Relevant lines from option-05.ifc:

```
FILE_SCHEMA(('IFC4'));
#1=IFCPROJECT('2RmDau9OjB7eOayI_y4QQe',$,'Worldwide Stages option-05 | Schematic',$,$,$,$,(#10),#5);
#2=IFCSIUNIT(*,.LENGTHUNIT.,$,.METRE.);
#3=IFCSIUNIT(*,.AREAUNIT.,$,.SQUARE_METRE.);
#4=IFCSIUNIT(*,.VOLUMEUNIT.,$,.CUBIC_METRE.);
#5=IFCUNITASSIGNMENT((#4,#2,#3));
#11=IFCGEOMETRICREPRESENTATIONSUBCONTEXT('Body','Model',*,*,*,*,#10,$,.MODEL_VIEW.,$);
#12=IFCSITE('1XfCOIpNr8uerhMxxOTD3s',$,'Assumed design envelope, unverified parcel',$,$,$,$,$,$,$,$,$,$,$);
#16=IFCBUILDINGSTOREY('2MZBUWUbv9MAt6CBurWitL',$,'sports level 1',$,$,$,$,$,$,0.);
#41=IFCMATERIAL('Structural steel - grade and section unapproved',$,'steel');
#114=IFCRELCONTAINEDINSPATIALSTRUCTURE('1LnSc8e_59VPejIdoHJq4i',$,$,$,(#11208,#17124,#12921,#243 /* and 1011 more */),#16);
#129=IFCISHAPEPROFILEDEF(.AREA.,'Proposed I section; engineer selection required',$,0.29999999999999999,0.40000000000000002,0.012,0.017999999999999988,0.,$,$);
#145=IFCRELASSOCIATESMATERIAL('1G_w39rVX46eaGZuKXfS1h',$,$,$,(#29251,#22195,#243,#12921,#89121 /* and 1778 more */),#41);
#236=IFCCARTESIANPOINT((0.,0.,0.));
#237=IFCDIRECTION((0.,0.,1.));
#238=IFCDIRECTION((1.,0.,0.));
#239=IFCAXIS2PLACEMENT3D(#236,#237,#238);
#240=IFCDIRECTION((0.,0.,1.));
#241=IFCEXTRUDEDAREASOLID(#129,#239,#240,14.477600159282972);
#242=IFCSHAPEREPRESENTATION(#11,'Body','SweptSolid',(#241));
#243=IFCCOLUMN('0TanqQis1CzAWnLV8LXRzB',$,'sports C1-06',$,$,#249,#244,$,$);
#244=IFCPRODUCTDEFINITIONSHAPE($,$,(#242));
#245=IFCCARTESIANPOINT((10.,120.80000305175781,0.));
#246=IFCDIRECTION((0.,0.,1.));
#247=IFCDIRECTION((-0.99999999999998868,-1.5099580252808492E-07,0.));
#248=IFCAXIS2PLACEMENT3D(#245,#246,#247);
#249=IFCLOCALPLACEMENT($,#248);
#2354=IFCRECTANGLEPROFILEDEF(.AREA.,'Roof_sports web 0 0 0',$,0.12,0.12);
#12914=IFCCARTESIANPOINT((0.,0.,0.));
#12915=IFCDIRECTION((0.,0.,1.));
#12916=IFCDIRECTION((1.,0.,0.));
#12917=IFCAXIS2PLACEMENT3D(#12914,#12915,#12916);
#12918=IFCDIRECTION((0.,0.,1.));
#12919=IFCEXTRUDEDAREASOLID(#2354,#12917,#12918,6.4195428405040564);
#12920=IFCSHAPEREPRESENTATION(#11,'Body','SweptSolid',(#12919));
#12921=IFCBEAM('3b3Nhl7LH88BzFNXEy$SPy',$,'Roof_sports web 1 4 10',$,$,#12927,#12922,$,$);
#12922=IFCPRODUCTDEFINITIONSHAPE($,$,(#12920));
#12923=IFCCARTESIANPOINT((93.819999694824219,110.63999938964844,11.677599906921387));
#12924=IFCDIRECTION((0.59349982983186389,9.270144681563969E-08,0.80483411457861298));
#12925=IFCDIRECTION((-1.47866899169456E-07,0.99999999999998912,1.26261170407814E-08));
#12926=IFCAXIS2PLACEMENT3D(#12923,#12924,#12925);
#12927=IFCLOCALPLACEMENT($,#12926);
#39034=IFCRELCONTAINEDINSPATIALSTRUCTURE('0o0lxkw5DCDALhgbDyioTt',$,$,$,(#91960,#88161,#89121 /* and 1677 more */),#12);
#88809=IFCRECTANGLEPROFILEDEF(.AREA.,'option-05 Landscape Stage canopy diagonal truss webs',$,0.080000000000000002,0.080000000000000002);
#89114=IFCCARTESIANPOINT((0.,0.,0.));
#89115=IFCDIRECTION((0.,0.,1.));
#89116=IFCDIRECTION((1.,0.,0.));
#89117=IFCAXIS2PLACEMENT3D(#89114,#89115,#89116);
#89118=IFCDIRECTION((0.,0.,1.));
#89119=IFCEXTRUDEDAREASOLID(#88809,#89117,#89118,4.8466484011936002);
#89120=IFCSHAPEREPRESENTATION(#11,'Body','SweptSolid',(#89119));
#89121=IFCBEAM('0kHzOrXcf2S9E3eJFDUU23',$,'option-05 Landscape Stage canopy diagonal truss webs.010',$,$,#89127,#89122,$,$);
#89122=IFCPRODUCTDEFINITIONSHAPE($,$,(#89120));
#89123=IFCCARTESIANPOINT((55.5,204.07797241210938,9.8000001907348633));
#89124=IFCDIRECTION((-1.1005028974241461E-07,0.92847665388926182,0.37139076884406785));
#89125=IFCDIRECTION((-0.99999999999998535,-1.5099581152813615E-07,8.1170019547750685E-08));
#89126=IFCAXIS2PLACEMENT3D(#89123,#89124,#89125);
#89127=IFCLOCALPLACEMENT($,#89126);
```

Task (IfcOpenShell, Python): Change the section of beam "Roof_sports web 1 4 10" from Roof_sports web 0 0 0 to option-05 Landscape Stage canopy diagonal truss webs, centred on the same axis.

```python
import ifcopenshell
import ifcopenshell.util.element
import ifcopenshell.util.representation

model = ifcopenshell.open("option-05.ifc")

member = model.by_guid("3b3Nhl7LH88BzFNXEy$SPy")
source = next(p for p in model.by_type("IfcRectangleProfileDef") if p.ProfileName == "option-05 Landscape Stage canopy diagonal truss webs")

body = ifcopenshell.util.representation.get_representation(member, "Model", "Body")
solid = body.Items[0]
old_profile = solid.SweptArea

# Copy the section's sizes but keep this member's own profile position.
profile = ifcopenshell.util.element.copy(model, source)
profile.Position = old_profile.Position
solid.SweptArea = profile
if not model.get_total_inverses(old_profile):
    ifcopenshell.util.element.remove_deep2(model, old_profile)

print(solid.SweptArea)

model.write("option-05_v2.ifc")
```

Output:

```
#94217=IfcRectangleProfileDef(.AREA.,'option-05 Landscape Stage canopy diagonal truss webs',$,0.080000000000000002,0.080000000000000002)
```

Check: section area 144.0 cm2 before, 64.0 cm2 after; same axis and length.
